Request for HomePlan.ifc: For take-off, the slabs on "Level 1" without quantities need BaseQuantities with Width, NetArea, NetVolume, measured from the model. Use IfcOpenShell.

First a look at what the model holds.

```python
import ifcopenshell
import ifcopenshell.util.element
import ifcopenshell.util.unit

model = ifcopenshell.open("HomePlan.ifc")
print(model.schema)
for unit_type in ("LENGTHUNIT", "AREAUNIT", "VOLUMEUNIT"):
    print(unit_type, ifcopenshell.util.unit.calculate_unit_scale(model, unit_type))
storey = next(s for s in model.by_type("IfcBuildingStorey") if s.Name == "Level 1")
slabs = [e for e in ifcopenshell.util.element.get_decomposition(storey) if e.is_a("IfcSlab")]
for e in sorted(slabs, key=lambda e: e.id()):
    print(e.id(), e.is_a(), e.Name, list(ifcopenshell.util.element.get_psets(e, qtos_only=True)), sep=" | ")
```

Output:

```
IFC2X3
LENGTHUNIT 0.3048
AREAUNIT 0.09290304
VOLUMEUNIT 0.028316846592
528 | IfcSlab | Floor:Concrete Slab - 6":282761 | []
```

```python
import ifcopenshell
import ifcopenshell.api.pset
import ifcopenshell.geom
import ifcopenshell.util.element
import ifcopenshell.util.shape
import ifcopenshell.util.unit

model = ifcopenshell.open("HomePlan.ifc")
unit_scale = ifcopenshell.util.unit.calculate_unit_scale(model)
area_scale = ifcopenshell.util.unit.calculate_unit_scale(model, "AREAUNIT")
volume_scale = ifcopenshell.util.unit.calculate_unit_scale(model, "VOLUMEUNIT")
settings = ifcopenshell.geom.settings()

storey = next(s for s in model.by_type("IfcBuildingStorey") if s.Name == "Level 1")
slabs = [e for e in ifcopenshell.util.element.get_decomposition(storey) if e.is_a("IfcSlab")]

for e in sorted(slabs, key=lambda e: e.id()):
    if ifcopenshell.util.element.get_psets(e, qtos_only=True, should_inherit=False):
        continue
    # Geometry comes back in metres, in the element's own axes.
    shape = ifcopenshell.geom.create_shape(settings, e)
    values = {
        "Width": ifcopenshell.util.shape.get_z(shape.geometry) / unit_scale,
        "NetArea": ifcopenshell.util.shape.get_footprint_area(shape.geometry) / area_scale,
        "NetVolume": ifcopenshell.util.shape.get_volume(shape.geometry) / volume_scale,
    }
    qto = ifcopenshell.api.pset.add_qto(model, product=e, name="BaseQuantities")
    ifcopenshell.api.pset.edit_qto(model, qto=qto, properties=values)
    print(e.id(), {k: round(v, 3) for k, v in values.items()})

model.write("HomePlan_rev.ifc")
```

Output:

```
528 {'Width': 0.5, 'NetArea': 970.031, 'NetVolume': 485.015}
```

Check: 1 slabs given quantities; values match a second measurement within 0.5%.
